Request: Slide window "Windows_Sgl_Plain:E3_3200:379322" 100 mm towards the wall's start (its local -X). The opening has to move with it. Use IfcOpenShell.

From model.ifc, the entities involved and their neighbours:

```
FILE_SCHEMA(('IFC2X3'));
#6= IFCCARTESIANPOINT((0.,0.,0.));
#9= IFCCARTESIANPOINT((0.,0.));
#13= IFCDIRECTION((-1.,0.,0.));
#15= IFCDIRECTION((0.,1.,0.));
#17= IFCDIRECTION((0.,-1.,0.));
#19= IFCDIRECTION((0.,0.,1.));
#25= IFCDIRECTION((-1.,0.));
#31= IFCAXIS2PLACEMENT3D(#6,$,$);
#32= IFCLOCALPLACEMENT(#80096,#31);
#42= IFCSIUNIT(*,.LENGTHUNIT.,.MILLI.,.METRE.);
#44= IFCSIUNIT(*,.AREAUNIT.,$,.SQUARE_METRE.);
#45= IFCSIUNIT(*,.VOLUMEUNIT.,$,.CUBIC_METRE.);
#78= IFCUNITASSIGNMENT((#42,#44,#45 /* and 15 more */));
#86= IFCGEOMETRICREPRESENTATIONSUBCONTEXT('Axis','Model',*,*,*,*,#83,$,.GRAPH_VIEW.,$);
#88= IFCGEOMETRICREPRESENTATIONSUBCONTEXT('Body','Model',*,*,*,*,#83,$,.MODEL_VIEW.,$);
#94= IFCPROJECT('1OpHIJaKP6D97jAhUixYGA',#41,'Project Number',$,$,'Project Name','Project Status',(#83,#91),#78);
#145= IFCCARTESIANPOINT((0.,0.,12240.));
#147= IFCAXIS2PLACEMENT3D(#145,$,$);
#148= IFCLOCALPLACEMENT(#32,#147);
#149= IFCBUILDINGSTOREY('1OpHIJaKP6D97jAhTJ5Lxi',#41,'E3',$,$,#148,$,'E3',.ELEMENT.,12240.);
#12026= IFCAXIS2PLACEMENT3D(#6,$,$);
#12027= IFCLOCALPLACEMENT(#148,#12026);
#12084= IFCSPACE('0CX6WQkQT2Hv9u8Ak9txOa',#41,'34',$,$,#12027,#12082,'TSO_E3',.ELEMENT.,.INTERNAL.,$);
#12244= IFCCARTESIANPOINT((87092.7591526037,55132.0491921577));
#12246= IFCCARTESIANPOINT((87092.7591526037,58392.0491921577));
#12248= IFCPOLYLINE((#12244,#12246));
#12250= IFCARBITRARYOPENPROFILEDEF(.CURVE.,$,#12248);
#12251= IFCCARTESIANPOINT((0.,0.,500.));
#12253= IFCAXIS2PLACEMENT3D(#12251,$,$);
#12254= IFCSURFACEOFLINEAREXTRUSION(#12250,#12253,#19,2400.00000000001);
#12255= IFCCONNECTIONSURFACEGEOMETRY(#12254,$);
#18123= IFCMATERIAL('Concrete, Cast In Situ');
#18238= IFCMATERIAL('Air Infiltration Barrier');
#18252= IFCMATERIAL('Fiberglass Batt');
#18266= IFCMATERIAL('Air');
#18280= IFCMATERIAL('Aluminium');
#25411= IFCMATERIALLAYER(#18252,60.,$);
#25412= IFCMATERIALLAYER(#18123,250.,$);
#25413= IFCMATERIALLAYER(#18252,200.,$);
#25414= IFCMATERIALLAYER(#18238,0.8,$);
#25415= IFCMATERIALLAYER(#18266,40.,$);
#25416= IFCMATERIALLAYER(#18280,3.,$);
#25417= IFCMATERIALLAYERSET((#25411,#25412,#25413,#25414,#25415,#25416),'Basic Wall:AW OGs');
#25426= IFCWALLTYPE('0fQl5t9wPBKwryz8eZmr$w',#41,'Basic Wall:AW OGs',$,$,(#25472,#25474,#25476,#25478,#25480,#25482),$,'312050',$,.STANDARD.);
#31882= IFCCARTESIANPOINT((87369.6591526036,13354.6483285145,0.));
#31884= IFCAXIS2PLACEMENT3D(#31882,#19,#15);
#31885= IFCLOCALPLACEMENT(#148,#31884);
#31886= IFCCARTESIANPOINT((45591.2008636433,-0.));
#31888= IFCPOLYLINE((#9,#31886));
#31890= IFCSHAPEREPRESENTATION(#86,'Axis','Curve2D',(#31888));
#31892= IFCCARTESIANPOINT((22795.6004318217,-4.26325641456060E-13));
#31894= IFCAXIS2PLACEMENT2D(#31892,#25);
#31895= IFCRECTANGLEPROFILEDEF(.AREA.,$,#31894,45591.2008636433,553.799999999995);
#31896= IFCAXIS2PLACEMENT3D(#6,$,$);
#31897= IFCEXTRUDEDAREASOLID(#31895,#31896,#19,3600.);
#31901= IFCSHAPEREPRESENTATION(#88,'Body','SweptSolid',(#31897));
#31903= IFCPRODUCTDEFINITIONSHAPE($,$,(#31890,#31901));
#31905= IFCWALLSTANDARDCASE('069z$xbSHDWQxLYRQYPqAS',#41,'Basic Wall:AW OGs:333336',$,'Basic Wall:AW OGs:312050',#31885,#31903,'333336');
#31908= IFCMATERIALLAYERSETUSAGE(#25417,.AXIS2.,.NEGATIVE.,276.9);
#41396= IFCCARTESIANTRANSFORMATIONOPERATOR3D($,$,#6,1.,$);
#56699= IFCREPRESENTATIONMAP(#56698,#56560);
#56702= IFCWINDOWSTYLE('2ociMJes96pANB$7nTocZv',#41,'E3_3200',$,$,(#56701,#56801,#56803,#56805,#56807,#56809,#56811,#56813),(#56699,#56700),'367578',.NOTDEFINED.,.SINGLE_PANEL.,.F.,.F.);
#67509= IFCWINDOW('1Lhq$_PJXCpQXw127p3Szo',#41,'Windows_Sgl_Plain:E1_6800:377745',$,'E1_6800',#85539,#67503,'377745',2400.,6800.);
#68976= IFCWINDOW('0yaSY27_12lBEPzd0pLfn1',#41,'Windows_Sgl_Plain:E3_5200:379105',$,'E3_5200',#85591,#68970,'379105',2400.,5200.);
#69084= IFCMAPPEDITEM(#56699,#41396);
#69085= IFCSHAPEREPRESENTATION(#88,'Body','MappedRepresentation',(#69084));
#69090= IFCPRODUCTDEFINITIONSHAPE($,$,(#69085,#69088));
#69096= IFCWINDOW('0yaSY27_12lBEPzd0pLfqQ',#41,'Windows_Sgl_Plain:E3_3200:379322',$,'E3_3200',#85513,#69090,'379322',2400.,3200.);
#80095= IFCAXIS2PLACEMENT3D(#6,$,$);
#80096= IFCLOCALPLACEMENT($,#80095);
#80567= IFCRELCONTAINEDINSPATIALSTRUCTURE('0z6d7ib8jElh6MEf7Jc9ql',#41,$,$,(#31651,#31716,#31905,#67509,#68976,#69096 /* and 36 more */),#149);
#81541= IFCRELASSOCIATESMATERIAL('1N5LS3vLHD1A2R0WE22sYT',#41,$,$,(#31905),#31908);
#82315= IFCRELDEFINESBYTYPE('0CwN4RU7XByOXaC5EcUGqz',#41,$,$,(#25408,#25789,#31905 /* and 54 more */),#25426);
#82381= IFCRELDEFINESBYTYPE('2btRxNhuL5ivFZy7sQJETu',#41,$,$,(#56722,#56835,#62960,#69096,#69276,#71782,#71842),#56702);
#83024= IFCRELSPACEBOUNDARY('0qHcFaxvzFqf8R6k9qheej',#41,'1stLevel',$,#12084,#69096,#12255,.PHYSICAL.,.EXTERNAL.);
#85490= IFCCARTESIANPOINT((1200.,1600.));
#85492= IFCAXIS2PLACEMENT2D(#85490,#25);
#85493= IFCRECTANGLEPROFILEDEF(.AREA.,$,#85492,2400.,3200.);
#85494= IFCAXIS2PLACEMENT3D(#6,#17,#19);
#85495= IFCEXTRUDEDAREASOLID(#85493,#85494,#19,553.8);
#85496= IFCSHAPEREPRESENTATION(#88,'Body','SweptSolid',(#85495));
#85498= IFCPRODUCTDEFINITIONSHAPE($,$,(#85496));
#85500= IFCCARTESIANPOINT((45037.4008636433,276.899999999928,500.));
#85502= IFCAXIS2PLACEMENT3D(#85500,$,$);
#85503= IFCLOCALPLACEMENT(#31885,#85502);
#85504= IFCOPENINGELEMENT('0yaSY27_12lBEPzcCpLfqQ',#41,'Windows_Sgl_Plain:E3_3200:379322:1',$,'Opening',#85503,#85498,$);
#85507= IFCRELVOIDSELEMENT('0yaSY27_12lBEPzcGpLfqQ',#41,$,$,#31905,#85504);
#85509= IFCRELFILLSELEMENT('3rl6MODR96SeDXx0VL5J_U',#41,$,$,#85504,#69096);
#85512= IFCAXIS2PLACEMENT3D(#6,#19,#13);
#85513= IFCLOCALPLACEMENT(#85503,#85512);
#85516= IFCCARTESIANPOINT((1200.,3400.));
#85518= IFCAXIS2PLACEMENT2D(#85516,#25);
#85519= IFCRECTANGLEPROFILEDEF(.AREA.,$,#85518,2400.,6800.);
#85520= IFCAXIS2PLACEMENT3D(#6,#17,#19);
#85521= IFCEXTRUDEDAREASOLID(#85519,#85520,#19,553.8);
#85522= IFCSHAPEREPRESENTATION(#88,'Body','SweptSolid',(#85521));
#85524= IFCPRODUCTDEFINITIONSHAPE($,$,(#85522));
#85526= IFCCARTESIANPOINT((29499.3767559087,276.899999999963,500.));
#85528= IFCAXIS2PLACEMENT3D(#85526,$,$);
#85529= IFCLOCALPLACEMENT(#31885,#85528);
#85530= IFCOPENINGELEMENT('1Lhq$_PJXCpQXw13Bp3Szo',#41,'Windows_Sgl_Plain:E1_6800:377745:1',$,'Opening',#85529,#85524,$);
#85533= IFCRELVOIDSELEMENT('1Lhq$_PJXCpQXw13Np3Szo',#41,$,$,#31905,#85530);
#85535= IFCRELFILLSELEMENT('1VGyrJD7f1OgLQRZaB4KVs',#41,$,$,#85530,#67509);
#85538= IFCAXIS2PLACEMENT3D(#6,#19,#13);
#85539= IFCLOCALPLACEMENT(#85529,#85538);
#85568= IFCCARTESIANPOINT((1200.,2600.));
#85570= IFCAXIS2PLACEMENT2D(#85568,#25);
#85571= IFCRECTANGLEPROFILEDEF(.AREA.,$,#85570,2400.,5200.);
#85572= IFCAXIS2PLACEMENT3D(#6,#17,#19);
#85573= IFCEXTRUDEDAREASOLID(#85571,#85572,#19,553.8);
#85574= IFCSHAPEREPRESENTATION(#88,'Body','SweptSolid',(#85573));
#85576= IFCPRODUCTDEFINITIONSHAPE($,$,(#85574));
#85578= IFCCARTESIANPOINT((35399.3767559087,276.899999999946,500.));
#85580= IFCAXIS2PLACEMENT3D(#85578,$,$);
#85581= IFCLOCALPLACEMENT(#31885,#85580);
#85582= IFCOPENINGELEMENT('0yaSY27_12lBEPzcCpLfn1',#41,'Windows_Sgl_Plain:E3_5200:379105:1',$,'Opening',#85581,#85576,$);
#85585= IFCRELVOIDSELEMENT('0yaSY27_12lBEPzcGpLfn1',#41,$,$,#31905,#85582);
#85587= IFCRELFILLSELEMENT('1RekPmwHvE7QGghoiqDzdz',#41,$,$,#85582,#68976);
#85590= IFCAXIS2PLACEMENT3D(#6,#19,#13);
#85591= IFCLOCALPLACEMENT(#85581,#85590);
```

```python
import numpy as np
import ifcopenshell
import ifcopenshell.api.geometry
import ifcopenshell.util.placement
import ifcopenshell.util.unit

model = ifcopenshell.open("model.ifc")
unit_scale = ifcopenshell.util.unit.calculate_unit_scale(model)

window = model.by_id(69096)
opening = window.FillsVoids[0].RelatingOpeningElement
wall = opening.VoidsElements[0].RelatingBuildingElement

wall_matrix = ifcopenshell.util.placement.get_local_placement(wall.ObjectPlacement)
shift = wall_matrix[:3, 0] * -0.1 / unit_scale
before = ifcopenshell.util.placement.get_local_placement(window.ObjectPlacement)[:3, 3].copy()

# The window is placed relative to its opening, so it follows when the opening moves.
matrix = ifcopenshell.util.placement.get_local_placement(opening.ObjectPlacement)
matrix[:3, 3] += shift
ifcopenshell.api.geometry.edit_object_placement(
    model, product=opening, matrix=matrix, is_si=False, should_transform_children=True
)

# Space boundary surfaces are stored in each space's coordinates; move them too.
for rel in window.ProvidesBoundaries:
    if not rel.ConnectionGeometry:
        continue
    surface = rel.ConnectionGeometry.SurfaceOnRelatingElement
    space_matrix = ifcopenshell.util.placement.get_local_placement(rel.RelatingSpace.ObjectPlacement)
    point = np.array(surface.Position.Location.Coordinates) + space_matrix[:3, :3].T @ shift
    surface.Position = model.createIfcAxis2Placement3D(
        model.createIfcCartesianPoint(point.tolist()), surface.Position.Axis, surface.Position.RefDirection
    )

after = ifcopenshell.util.placement.get_local_placement(window.ObjectPlacement)[:3, 3]
print("window moved by", (after - before).round(3) + 0.0)

model.write("model_v2.ifc")
```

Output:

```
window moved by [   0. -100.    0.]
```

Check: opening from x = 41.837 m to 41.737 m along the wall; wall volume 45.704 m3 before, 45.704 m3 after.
